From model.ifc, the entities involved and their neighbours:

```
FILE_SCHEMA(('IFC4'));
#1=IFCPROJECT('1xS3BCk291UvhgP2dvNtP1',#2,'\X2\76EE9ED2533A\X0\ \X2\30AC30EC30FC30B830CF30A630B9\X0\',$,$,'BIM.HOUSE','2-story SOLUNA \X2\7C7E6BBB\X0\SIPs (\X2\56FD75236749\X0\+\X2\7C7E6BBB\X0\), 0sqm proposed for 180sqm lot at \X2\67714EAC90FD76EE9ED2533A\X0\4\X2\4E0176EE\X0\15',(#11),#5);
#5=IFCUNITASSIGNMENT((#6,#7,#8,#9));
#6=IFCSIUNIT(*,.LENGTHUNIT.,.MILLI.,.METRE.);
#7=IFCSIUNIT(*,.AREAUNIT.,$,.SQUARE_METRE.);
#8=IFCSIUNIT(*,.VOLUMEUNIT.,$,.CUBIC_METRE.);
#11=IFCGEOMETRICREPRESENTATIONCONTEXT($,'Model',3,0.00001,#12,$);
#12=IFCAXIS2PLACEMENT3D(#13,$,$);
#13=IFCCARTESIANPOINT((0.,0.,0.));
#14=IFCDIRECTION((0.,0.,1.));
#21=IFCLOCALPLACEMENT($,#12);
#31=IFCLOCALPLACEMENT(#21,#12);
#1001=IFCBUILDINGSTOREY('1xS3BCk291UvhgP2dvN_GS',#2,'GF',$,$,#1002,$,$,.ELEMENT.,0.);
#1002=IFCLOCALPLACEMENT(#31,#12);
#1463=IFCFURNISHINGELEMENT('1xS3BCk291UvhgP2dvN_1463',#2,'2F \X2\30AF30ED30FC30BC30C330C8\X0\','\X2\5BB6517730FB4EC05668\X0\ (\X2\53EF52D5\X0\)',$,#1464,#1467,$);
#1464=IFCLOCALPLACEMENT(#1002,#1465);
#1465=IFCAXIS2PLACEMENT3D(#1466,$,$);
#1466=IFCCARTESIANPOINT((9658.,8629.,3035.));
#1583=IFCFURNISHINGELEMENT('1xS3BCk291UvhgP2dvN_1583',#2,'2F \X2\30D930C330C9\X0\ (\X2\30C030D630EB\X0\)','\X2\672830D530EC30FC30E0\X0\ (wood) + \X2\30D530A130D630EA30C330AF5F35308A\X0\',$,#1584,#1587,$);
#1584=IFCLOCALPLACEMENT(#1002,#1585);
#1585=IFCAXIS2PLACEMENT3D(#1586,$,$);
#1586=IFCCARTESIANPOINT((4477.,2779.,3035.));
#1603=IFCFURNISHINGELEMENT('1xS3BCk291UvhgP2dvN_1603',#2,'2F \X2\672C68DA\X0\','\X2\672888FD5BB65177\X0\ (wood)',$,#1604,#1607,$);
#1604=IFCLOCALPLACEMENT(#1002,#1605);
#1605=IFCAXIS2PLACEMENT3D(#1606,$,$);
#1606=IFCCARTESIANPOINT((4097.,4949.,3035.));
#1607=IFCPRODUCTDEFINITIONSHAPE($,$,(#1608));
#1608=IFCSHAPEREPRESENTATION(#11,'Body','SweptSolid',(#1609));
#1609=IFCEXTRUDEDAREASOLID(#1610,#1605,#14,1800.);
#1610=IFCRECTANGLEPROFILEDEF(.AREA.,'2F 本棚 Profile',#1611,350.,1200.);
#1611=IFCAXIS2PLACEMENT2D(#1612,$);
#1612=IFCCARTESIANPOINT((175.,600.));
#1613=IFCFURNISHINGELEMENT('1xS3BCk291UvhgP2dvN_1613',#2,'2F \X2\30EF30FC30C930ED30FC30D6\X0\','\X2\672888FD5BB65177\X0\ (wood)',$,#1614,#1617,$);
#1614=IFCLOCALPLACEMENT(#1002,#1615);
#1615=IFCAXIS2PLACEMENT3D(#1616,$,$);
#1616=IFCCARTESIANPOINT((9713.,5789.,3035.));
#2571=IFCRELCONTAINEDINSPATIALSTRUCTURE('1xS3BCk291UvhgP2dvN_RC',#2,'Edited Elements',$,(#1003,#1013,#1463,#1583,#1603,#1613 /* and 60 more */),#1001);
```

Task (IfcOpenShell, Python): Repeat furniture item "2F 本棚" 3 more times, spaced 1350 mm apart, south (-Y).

```python
import numpy as np
import ifcopenshell
import ifcopenshell.api.geometry
import ifcopenshell.api.root
import ifcopenshell.util.element
import ifcopenshell.util.placement
import ifcopenshell.util.unit

model = ifcopenshell.open("model.ifc")
unit_scale = ifcopenshell.util.unit.calculate_unit_scale(model)


def reuse_history(source, copy):
    """copy_class also copies each property set's owner history, people and application; keep the originals."""
    for rel in copy.IsDefinedBy:
        if rel.is_a("IfcRelDefinesByProperties") and (history := rel.RelatingPropertyDefinition.OwnerHistory):
            rel.RelatingPropertyDefinition.OwnerHistory = source.OwnerHistory
            ifcopenshell.util.element.remove_deep2(model, history)


source = model.by_id(1603)
base = ifcopenshell.util.placement.get_local_placement(source.ObjectPlacement)
step = np.array([0.0, -1.0, 0.0]) * 1.35 / unit_scale

for i in range(1, 4):
    copy = ifcopenshell.api.root.copy_class(model, product=source)
    copy.Representation = ifcopenshell.util.element.copy_deep(
        model, source.Representation, exclude=["IfcGeometricRepresentationContext", "IfcRepresentationMap"]
    )
    reuse_history(source, copy)
    matrix = base.copy()
    matrix[:3, 3] += i * step
    print("added at", matrix[:3, 3].round(3) + 0.0)
    ifcopenshell.api.geometry.edit_object_placement(model, product=copy, matrix=matrix, is_si=False)

model.write("model_updated.ifc")
```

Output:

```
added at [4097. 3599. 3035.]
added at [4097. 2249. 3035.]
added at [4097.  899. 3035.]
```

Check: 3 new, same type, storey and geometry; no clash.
